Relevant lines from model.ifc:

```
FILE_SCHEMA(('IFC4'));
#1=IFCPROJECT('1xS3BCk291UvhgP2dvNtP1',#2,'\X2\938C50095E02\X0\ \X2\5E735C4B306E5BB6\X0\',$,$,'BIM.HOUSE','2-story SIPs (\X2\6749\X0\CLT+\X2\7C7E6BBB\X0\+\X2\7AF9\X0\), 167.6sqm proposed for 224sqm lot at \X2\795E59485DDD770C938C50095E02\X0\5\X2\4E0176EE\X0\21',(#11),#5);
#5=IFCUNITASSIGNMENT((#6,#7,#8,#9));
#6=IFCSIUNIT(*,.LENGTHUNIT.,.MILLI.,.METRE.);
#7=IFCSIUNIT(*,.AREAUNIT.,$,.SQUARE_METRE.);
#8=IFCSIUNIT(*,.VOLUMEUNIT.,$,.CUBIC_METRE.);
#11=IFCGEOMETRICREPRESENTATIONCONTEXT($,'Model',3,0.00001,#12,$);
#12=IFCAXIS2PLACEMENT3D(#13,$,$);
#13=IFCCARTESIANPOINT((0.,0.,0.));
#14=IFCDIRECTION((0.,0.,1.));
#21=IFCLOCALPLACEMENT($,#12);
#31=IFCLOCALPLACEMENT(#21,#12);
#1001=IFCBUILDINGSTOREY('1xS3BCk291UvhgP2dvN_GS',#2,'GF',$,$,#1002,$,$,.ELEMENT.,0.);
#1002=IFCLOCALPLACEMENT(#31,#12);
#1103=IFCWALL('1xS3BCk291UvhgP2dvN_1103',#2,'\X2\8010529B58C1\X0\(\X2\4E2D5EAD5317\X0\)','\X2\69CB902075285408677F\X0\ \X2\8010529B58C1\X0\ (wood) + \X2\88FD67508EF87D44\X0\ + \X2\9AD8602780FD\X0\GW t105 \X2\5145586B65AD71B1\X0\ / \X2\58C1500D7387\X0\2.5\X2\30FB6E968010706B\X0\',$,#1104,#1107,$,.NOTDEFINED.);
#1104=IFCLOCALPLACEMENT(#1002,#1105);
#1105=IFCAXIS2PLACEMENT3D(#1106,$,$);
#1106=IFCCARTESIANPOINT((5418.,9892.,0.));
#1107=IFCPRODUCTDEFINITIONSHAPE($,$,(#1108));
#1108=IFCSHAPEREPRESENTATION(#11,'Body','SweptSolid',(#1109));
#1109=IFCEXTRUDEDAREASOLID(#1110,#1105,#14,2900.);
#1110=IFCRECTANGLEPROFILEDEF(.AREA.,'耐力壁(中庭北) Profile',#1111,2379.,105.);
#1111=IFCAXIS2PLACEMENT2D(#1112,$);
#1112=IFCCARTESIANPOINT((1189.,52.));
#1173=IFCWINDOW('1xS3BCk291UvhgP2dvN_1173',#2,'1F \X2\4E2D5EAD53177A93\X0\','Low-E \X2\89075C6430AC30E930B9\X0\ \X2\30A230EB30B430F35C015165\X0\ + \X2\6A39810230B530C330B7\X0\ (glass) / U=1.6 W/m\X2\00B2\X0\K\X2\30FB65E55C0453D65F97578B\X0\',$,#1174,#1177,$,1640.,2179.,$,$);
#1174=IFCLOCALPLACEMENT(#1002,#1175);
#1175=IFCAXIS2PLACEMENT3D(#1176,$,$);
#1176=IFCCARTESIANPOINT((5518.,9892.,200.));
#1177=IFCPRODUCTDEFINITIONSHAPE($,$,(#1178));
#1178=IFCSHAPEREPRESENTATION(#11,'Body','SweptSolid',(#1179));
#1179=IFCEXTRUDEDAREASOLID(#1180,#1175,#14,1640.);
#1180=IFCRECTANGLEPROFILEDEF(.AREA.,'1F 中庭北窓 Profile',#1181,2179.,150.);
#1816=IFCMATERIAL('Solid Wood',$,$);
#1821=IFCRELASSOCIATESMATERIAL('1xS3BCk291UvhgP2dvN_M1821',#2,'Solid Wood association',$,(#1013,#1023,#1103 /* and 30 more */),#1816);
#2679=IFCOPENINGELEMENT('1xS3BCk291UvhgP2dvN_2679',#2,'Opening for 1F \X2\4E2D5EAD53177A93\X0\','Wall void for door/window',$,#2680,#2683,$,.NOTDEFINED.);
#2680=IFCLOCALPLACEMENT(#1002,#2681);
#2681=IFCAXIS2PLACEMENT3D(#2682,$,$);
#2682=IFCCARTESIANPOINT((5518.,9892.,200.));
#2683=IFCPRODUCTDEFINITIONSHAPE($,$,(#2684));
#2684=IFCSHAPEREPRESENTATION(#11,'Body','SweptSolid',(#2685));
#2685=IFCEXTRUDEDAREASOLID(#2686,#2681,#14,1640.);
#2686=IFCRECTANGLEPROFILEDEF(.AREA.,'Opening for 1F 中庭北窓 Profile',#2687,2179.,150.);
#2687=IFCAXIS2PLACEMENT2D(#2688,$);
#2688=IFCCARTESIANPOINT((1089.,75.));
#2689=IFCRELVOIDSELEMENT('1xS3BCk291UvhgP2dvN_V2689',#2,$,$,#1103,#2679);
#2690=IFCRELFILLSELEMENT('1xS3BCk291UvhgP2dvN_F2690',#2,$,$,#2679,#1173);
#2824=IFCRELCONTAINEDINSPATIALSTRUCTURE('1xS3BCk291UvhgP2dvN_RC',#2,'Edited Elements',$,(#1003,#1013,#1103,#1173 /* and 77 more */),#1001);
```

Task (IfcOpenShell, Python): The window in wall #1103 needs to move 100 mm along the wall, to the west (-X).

```python
import ifcopenshell
import ifcopenshell.api.geometry
import ifcopenshell.util.placement
import ifcopenshell.util.unit

model = ifcopenshell.open("model.ifc")
unit_scale = ifcopenshell.util.unit.calculate_unit_scale(model)

window = model.by_guid("1xS3BCk291UvhgP2dvN_1173")
opening = window.FillsVoids[0].RelatingOpeningElement
wall = opening.VoidsElements[0].RelatingBuildingElement

wall_matrix = ifcopenshell.util.placement.get_local_placement(wall.ObjectPlacement)
shift = wall_matrix[:3, 0] * -0.1 / unit_scale
before = ifcopenshell.util.placement.get_local_placement(window.ObjectPlacement)[:3, 3].copy()

# The window is not placed relative to its opening, so move both.
for product in (opening, window):
    matrix = ifcopenshell.util.placement.get_local_placement(product.ObjectPlacement)
    matrix[:3, 3] += shift
    ifcopenshell.api.geometry.edit_object_placement(model, product=product, matrix=matrix, is_si=False)

after = ifcopenshell.util.placement.get_local_placement(window.ObjectPlacement)[:3, 3]
print("window moved by", (after - before).round(3) + 0.0)

model.write("model_updated.ifc")
```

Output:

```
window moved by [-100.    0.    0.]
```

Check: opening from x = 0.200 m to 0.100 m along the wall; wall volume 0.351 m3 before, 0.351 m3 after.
